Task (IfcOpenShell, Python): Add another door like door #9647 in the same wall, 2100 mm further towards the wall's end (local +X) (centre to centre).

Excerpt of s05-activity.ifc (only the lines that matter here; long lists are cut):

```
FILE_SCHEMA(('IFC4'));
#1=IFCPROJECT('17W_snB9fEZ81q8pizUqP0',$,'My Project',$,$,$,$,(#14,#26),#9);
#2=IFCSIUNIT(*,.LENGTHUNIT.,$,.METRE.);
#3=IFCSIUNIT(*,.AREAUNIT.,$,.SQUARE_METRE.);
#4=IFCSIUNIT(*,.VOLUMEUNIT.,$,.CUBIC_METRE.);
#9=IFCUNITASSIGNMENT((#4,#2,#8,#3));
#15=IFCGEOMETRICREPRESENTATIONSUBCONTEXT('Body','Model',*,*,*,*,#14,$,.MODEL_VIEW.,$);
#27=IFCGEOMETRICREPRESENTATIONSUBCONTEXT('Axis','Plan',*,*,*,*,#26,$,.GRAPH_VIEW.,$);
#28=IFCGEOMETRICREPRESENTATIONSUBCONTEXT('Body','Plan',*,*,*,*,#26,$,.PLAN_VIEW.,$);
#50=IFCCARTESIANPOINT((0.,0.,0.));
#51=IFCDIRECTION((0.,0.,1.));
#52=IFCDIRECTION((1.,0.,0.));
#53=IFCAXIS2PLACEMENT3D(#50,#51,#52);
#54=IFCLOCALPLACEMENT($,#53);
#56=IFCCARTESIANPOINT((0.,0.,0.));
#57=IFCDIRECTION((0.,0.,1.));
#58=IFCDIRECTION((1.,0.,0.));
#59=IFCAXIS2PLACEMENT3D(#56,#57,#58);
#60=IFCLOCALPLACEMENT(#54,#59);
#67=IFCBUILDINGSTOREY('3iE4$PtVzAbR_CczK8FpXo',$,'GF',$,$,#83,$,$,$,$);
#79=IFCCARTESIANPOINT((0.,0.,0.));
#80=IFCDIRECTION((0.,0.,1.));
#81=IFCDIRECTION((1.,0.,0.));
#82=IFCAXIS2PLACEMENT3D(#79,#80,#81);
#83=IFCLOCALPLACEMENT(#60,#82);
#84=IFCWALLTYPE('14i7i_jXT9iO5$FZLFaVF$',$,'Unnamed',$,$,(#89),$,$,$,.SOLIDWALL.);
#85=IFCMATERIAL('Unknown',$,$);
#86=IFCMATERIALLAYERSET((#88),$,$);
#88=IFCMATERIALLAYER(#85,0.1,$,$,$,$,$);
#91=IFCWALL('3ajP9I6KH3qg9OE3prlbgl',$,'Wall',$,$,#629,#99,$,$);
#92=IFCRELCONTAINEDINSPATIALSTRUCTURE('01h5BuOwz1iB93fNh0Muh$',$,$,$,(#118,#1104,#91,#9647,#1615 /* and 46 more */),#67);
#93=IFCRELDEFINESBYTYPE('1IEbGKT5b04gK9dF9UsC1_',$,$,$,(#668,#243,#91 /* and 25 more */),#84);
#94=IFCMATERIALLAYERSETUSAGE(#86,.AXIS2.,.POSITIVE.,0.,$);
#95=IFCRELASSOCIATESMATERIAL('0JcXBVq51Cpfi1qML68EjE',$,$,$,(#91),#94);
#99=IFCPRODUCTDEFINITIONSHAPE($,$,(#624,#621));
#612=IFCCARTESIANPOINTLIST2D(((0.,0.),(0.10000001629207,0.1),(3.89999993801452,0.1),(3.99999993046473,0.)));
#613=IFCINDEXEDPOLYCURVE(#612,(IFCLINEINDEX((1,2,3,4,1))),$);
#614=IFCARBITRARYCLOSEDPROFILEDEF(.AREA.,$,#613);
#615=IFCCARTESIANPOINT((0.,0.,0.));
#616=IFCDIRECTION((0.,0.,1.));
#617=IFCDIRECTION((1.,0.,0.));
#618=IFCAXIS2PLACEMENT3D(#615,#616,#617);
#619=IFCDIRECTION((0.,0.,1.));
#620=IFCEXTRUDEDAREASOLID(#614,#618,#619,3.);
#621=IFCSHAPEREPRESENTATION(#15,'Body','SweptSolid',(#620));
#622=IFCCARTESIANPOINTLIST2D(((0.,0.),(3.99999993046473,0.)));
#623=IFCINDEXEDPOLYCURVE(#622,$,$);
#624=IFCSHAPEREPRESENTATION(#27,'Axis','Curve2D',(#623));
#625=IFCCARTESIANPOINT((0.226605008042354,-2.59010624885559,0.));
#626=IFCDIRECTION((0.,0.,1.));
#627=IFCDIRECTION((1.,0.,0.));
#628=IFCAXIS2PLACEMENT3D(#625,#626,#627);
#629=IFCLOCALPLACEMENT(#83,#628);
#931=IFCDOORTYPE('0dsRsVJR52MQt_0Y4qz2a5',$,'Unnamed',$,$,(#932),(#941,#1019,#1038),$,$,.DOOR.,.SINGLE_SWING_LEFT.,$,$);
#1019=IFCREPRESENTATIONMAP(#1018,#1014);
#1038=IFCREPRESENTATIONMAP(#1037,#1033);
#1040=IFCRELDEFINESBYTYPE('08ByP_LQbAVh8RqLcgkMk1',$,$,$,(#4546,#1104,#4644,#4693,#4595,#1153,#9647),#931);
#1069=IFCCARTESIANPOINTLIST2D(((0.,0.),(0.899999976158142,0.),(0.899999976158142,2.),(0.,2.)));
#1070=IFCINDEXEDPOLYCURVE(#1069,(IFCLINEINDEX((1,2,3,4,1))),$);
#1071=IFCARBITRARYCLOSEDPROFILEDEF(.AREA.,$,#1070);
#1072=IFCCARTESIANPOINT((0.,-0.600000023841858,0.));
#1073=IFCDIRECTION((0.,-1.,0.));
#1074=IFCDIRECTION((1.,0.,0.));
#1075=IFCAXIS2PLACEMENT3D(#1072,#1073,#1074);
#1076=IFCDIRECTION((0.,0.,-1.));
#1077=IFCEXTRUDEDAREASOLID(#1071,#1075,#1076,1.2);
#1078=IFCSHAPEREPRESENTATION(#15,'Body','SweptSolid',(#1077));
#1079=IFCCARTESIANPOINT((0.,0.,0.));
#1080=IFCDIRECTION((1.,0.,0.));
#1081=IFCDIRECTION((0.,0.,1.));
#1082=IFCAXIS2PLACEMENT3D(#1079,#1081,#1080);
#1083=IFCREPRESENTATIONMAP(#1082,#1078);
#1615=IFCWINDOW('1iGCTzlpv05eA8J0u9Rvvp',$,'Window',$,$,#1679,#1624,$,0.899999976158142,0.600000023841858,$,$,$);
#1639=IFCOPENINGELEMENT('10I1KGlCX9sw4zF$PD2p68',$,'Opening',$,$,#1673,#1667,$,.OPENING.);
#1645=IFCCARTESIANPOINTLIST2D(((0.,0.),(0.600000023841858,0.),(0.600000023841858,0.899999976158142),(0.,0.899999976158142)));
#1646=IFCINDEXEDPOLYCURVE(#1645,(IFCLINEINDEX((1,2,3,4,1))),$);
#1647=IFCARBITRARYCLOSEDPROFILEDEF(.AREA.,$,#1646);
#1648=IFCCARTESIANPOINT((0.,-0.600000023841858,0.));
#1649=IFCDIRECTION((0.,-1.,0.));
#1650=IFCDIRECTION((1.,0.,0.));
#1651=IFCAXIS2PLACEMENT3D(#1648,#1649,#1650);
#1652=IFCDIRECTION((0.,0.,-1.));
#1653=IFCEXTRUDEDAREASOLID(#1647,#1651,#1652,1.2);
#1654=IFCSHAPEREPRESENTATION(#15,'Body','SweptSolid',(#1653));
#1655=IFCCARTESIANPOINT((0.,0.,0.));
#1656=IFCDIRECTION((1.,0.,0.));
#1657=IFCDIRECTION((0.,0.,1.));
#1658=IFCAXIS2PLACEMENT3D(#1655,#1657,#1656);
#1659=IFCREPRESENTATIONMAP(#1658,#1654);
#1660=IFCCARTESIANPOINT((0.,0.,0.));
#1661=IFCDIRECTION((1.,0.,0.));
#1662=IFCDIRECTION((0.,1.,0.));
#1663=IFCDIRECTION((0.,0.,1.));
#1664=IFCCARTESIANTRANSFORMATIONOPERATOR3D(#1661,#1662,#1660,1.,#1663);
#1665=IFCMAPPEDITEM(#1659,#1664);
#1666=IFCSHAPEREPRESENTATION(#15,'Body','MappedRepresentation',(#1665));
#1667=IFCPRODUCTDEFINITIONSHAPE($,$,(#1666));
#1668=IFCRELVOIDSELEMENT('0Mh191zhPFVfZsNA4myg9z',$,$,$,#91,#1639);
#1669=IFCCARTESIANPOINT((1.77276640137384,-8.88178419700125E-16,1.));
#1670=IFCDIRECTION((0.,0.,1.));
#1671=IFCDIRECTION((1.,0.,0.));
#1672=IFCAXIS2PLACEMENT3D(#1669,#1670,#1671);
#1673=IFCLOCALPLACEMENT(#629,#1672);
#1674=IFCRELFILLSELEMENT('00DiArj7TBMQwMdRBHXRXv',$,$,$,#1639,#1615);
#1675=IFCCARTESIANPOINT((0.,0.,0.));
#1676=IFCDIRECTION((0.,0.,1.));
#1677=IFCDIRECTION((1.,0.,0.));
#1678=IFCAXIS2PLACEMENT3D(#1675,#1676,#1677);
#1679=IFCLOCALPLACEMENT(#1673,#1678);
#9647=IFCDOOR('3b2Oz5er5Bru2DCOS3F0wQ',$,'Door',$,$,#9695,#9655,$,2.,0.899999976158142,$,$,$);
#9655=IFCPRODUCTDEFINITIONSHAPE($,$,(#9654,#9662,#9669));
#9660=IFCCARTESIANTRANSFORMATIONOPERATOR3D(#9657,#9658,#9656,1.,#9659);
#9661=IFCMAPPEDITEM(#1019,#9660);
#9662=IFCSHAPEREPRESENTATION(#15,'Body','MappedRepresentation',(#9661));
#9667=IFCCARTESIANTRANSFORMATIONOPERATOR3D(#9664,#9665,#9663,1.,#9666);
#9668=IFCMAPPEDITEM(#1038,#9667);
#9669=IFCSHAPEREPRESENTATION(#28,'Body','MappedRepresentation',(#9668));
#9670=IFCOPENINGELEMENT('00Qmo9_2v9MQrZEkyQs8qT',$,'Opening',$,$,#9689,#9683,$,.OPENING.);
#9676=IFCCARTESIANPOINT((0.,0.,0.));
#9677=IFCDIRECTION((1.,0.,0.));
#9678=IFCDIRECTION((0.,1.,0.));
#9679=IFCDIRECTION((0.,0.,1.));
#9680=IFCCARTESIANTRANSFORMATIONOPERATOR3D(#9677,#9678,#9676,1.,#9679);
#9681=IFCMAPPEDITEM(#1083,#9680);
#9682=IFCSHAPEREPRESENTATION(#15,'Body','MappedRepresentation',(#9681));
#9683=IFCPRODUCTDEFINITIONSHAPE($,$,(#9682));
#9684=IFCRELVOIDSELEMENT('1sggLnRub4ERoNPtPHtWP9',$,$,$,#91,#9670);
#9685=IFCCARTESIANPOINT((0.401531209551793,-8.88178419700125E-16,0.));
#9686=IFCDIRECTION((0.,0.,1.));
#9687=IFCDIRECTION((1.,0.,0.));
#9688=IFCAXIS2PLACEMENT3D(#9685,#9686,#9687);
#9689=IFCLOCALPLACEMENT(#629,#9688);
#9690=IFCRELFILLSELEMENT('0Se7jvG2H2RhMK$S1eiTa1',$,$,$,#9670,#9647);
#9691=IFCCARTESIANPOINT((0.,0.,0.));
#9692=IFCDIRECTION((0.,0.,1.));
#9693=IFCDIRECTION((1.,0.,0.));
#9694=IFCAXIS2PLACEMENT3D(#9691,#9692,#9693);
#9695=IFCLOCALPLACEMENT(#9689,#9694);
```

```python
import ifcopenshell
import ifcopenshell.api.feature
import ifcopenshell.api.geometry
import ifcopenshell.api.root
import ifcopenshell.geom
import ifcopenshell.util.element
import ifcopenshell.util.placement
import ifcopenshell.util.shape

model = ifcopenshell.open("s05-activity.ifc")
settings = ifcopenshell.geom.settings()


def volume(element):
    """Net volume in cubic metres, openings subtracted."""
    shape = ifcopenshell.geom.create_shape(settings, element)
    return ifcopenshell.util.shape.get_volume(shape.geometry)


door = model.by_id(9647)
opening = door.FillsVoids[0].RelatingOpeningElement
wall = opening.VoidsElements[0].RelatingBuildingElement
before = volume(wall)
shift = ifcopenshell.util.placement.get_local_placement(wall.ObjectPlacement)[:3, 0] * 2.1

# copy_class copies the void relationship, type, container and properties, but no geometry.
new_opening = ifcopenshell.api.root.copy_class(model, product=opening)
new_opening.Representation = ifcopenshell.util.element.copy_deep(
    model, opening.Representation, exclude=["IfcGeometricRepresentationContext", "IfcRepresentationMap"]
)
new_door = ifcopenshell.api.root.copy_class(model, product=door)
new_door.Representation = ifcopenshell.util.element.copy_deep(
    model, door.Representation, exclude=["IfcGeometricRepresentationContext", "IfcRepresentationMap"]
)
ifcopenshell.api.feature.add_filling(model, opening=new_opening, element=new_door)

for old, new in ((opening, new_opening), (door, new_door)):
    matrix = ifcopenshell.util.placement.get_local_placement(old.ObjectPlacement)
    matrix[:3, 3] += shift
    ifcopenshell.api.geometry.edit_object_placement(model, product=new, matrix=matrix, is_si=False)

after = volume(wall)

print(f"wall volume {before:.3f} -> {after:.3f} m3")

model.write("s05-activity_rev.ifc")
```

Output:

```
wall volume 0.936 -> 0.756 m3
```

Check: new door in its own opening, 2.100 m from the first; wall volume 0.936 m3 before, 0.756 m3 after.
